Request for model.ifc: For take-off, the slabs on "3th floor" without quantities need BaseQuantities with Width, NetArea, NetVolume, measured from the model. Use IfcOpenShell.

First a look at what the model holds.

```python
import ifcopenshell
import ifcopenshell.util.element
import ifcopenshell.util.unit

model = ifcopenshell.open("model.ifc")
print(model.schema)
for unit_type in ("LENGTHUNIT", "AREAUNIT", "VOLUMEUNIT"):
    print(unit_type, ifcopenshell.util.unit.calculate_unit_scale(model, unit_type))
storey = next(s for s in model.by_type("IfcBuildingStorey") if s.Name == "3th floor")
slabs = [e for e in ifcopenshell.util.element.get_decomposition(storey) if e.is_a("IfcSlab")]
for e in sorted(slabs, key=lambda e: e.id()):
    print(e.id(), e.is_a(), e.Name, list(ifcopenshell.util.element.get_psets(e, qtos_only=True)), sep=" | ")
```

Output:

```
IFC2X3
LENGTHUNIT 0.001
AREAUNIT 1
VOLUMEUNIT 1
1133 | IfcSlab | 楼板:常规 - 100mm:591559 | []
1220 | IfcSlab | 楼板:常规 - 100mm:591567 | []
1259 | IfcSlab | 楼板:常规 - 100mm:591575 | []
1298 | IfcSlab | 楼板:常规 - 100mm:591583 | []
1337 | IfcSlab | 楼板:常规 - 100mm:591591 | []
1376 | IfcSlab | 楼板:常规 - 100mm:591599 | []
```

```python
import ifcopenshell
import ifcopenshell.api.pset
import ifcopenshell.geom
import ifcopenshell.util.element
import ifcopenshell.util.shape
import ifcopenshell.util.unit

model = ifcopenshell.open("model.ifc")
unit_scale = ifcopenshell.util.unit.calculate_unit_scale(model)
area_scale = ifcopenshell.util.unit.calculate_unit_scale(model, "AREAUNIT")
volume_scale = ifcopenshell.util.unit.calculate_unit_scale(model, "VOLUMEUNIT")
settings = ifcopenshell.geom.settings()

storey = next(s for s in model.by_type("IfcBuildingStorey") if s.Name == "3th floor")
slabs = [e for e in ifcopenshell.util.element.get_decomposition(storey) if e.is_a("IfcSlab")]

for e in sorted(slabs, key=lambda e: e.id()):
    if ifcopenshell.util.element.get_psets(e, qtos_only=True, should_inherit=False):
        continue
    # Geometry comes back in metres, in the element's own axes.
    shape = ifcopenshell.geom.create_shape(settings, e)
    values = {
        "Width": ifcopenshell.util.shape.get_z(shape.geometry) / unit_scale,
        "NetArea": ifcopenshell.util.shape.get_footprint_area(shape.geometry) / area_scale,
        "NetVolume": ifcopenshell.util.shape.get_volume(shape.geometry) / volume_scale,
    }
    qto = ifcopenshell.api.pset.add_qto(model, product=e, name="BaseQuantities")
    ifcopenshell.api.pset.edit_qto(model, qto=qto, properties=values)
    print(e.id(), {k: round(v, 3) for k, v in values.items()})

model.write("model_v2.ifc")
```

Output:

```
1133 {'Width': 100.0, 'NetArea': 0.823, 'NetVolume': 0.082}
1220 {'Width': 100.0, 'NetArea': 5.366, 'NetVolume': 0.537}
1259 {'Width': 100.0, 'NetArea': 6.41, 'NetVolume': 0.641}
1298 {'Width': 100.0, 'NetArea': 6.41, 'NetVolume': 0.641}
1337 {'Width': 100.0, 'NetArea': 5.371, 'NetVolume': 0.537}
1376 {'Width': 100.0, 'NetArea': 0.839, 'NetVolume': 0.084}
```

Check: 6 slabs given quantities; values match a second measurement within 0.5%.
